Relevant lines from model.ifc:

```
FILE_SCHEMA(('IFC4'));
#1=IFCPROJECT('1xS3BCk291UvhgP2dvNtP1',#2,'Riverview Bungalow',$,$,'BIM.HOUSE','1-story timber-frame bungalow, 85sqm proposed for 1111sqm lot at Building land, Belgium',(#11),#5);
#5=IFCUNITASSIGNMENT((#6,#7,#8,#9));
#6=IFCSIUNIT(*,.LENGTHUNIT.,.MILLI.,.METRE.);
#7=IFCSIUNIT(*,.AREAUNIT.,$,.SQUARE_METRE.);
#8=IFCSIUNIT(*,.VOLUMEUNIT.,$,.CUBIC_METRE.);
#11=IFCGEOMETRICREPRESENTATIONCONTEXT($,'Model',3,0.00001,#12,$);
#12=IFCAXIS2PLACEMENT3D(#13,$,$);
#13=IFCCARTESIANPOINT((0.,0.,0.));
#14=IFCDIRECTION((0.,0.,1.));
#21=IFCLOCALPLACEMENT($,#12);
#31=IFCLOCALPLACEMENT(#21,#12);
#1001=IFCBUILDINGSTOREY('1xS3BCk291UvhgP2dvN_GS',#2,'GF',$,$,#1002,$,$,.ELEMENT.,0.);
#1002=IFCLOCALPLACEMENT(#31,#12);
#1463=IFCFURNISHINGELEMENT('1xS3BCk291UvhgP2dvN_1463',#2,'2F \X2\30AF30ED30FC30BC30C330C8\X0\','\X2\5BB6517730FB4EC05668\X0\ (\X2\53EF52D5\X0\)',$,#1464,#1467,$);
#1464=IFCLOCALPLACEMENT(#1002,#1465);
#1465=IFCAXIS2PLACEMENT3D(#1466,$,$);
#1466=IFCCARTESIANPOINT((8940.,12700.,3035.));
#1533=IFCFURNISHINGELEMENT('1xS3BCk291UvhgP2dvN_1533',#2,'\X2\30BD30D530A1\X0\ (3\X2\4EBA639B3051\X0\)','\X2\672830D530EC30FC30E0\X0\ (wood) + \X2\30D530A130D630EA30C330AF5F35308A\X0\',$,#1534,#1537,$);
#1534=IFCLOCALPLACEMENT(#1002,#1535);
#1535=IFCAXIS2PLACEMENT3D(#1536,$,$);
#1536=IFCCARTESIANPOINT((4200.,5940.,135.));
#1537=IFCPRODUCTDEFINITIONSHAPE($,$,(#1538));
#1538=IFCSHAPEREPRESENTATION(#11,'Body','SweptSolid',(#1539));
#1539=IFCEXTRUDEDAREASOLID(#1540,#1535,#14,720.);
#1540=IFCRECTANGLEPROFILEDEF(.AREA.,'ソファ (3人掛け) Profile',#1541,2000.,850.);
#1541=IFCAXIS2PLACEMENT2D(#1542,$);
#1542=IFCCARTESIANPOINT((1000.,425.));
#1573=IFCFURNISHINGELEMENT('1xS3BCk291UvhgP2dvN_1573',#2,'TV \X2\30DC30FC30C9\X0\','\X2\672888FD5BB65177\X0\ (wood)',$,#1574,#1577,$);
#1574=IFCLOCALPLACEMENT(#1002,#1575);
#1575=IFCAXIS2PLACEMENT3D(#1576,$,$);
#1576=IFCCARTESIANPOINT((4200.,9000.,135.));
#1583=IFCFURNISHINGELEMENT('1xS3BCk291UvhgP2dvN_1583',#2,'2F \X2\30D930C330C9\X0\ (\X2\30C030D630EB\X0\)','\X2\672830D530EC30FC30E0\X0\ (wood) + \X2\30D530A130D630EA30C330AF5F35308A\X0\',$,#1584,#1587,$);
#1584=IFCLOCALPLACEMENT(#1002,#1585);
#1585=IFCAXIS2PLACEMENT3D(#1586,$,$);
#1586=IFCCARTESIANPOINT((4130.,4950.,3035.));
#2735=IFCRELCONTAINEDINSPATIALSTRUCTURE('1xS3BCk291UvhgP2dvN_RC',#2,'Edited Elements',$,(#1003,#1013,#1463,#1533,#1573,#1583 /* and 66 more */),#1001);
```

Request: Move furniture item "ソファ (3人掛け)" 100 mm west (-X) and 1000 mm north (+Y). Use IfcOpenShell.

```python
import ifcopenshell
import ifcopenshell.api.geometry
import ifcopenshell.util.placement
import ifcopenshell.util.unit

model = ifcopenshell.open("model.ifc")
unit_scale = ifcopenshell.util.unit.calculate_unit_scale(model)

item = model.by_guid("1xS3BCk291UvhgP2dvN_1533")
matrix = ifcopenshell.util.placement.get_local_placement(item.ObjectPlacement)
matrix[0, 3] -= 0.1 / unit_scale
matrix[1, 3] += 1 / unit_scale
ifcopenshell.api.geometry.edit_object_placement(model, product=item, matrix=matrix, is_si=False)

print(ifcopenshell.util.placement.get_local_placement(item.ObjectPlacement).round(3) + 0.0)

model.write("model_v2.ifc")
```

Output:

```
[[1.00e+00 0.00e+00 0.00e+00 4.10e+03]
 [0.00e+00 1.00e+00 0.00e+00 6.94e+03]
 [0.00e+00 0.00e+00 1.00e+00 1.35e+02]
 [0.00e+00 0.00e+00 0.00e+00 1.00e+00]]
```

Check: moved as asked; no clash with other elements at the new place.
